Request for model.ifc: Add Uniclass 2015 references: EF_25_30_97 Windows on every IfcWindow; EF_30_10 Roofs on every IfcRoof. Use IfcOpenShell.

First a look at what the model holds.

```python
import ifcopenshell

model = ifcopenshell.open("model.ifc")
print(model.schema)
print("classifications:", [c.Name for c in model.by_type("IfcClassification")])
for ifc_class in ("IfcDoor", "IfcRoof", "IfcStair", "IfcWall", "IfcWindow"):
    print(ifc_class, len(model.by_type(ifc_class)))
```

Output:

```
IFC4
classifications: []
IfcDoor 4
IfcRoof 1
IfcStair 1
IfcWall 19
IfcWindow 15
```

```python
import ifcopenshell
import ifcopenshell.api.classification

model = ifcopenshell.open("model.ifc")

system = ifcopenshell.api.classification.add_classification(model, classification="Uniclass 2015")

codes = {
    "IfcWindow": ("EF_25_30_97", "Windows"),
    "IfcRoof": ("EF_30_10", "Roofs"),
}
for ifc_class, (code, name) in codes.items():
    products = model.by_type(ifc_class)
    ifcopenshell.api.classification.add_reference(
        model, products=products, classification=system, identification=code, name=name
    )
    print(code, len(products))

model.write("model_edited.ifc")
```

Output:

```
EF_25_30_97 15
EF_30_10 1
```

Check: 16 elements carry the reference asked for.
